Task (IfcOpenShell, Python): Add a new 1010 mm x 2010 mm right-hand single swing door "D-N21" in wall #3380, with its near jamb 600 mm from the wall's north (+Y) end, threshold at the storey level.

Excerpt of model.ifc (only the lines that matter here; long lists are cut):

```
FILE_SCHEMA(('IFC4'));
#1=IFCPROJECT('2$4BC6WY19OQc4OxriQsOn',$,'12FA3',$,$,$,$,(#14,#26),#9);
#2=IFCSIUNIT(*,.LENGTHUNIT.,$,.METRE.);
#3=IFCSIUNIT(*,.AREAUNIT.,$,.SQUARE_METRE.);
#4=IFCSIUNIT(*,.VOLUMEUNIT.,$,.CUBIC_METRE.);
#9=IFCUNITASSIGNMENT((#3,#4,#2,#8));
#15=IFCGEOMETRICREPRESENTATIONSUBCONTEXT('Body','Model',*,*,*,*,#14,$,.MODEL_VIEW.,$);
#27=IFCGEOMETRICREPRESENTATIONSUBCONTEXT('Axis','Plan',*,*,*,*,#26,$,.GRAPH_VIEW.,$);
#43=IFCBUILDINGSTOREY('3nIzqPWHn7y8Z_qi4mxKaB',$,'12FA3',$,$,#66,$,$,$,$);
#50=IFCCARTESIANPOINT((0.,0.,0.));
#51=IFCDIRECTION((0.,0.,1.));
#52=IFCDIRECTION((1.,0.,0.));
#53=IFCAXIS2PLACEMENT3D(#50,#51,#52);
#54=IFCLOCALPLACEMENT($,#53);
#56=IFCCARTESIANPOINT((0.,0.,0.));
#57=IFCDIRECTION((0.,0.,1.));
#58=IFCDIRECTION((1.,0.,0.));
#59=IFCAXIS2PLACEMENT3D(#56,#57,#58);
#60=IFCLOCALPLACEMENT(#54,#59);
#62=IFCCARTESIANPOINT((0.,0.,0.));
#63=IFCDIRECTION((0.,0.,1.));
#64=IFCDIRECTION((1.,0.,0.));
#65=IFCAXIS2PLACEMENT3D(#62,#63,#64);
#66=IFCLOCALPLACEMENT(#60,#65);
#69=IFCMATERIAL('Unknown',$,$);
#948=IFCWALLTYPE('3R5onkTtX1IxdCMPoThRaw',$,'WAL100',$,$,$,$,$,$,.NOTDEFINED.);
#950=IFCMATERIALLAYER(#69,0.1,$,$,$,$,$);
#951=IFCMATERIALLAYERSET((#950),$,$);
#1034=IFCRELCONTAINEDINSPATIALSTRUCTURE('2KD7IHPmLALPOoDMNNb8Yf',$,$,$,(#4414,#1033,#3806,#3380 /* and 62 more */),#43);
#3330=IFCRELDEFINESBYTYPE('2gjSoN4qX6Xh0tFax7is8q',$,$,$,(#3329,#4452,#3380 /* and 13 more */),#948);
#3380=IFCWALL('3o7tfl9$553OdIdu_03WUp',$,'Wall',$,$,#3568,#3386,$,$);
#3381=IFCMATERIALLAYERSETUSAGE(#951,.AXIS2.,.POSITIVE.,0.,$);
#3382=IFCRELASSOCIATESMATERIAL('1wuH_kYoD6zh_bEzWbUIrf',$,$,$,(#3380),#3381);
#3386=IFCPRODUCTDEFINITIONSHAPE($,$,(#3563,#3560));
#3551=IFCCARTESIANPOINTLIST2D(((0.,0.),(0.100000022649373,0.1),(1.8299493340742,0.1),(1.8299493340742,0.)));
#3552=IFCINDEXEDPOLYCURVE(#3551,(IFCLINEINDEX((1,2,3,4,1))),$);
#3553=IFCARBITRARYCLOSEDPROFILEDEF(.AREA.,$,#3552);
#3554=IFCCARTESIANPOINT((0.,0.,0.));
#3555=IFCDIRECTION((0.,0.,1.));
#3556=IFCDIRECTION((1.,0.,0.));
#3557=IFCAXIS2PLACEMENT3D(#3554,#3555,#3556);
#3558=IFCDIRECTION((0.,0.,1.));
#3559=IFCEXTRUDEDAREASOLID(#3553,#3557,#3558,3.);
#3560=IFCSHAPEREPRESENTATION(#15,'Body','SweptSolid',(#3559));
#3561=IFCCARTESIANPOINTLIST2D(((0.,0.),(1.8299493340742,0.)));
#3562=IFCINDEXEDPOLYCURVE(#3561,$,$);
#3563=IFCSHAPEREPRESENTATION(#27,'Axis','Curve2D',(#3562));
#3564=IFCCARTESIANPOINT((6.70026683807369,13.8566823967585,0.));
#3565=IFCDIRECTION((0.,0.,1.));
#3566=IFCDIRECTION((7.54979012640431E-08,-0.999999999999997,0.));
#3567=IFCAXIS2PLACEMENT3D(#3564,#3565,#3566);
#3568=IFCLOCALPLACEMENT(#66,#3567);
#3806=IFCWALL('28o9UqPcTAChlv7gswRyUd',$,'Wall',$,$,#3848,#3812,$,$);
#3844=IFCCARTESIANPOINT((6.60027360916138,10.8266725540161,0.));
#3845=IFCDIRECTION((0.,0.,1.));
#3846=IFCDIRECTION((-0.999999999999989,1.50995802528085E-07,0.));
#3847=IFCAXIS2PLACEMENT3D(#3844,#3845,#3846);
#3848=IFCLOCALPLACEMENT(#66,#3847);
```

```python
import numpy as np
import ifcopenshell
import ifcopenshell.api.feature
import ifcopenshell.api.geometry
import ifcopenshell.api.root
import ifcopenshell.api.spatial
import ifcopenshell.geom
import ifcopenshell.util.element
import ifcopenshell.util.placement
import ifcopenshell.util.representation
import ifcopenshell.util.shape
import ifcopenshell.util.unit

model = ifcopenshell.open("model.ifc")
unit_scale = ifcopenshell.util.unit.calculate_unit_scale(model)
settings = ifcopenshell.geom.settings()


def volume(element):
    """Net volume in cubic metres, openings subtracted."""
    shape = ifcopenshell.geom.create_shape(settings, element)
    return ifcopenshell.util.shape.get_volume(shape.geometry)


wall = model.by_guid("3o7tfl9$553OdIdu_03WUp")
storey = ifcopenshell.util.element.get_container(wall, ifc_class="IfcBuildingStorey")
context = ifcopenshell.util.representation.get_context(model, "Model", "Body", "MODEL_VIEW")
before = volume(wall)

width, height, from_end, sill = 1.01, 2.01, 0.6, 0.0  # metres

# The wall runs along its own X axis, and the end named is its -X end.
wall_shape = ifcopenshell.geom.create_shape(settings, wall)
x, y, z = ifcopenshell.util.shape.get_vertices(wall_shape.geometry).T
start = x.min() + from_end
face, thickness = float(y.min()), float(y.max() - y.min())
wall_matrix = ifcopenshell.util.placement.get_local_placement(wall.ObjectPlacement)
level = ifcopenshell.util.placement.get_local_placement(storey.ObjectPlacement)[2, 3]


def in_wall(x, y):
    """Placement at x, y metres in the wall's axes, at sill height."""
    matrix = wall_matrix.copy()
    matrix[:, 3] = wall_matrix @ np.array([x / unit_scale, y / unit_scale, 0.0, 1.0])
    matrix[2, 3] = level + sill / unit_scale
    return matrix


# Opening: a box that overshoots both wall faces by 50 mm.
opening = ifcopenshell.api.root.create_entity(model, ifc_class="IfcOpeningElement", predefined_type="OPENING")
box = ifcopenshell.api.geometry.add_wall_representation(
    model, context=context, length=width, height=height, thickness=thickness + 0.1
)
ifcopenshell.api.geometry.assign_representation(model, product=opening, representation=box)
ifcopenshell.api.geometry.edit_object_placement(model, product=opening, matrix=in_wall(start, face - 0.05), is_si=False)
ifcopenshell.api.feature.add_feature(model, feature=opening, element=wall)

door = ifcopenshell.api.root.create_entity(model, ifc_class="IfcDoor", name="D-N21", predefined_type="DOOR")
door.OverallWidth, door.OverallHeight = width / unit_scale, height / unit_scale
door.OperationType = "SINGLE_SWING_RIGHT"
body = ifcopenshell.api.geometry.add_door_representation(
    model,
    context=context,
    overall_width=door.OverallWidth,
    overall_height=door.OverallHeight,
    operation_type="SINGLE_SWING_RIGHT",
    lining_properties={"LiningDepth": thickness / unit_scale, "ThresholdDepth": thickness / unit_scale},
)
ifcopenshell.api.geometry.assign_representation(model, product=door, representation=body)
ifcopenshell.api.spatial.assign_container(model, products=[door], relating_structure=storey)
ifcopenshell.api.feature.add_filling(model, opening=opening, element=door)

# The lining spans the wall, so the door starts at the wall face.
ifcopenshell.api.geometry.edit_object_placement(model, product=door, matrix=in_wall(start, face), is_si=False)

after = volume(wall)

print(f"wall volume {before:.3f} -> {after:.3f} m3")

model.write("model_updated.ifc")
```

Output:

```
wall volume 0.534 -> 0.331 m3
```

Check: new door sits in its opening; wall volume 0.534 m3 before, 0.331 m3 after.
